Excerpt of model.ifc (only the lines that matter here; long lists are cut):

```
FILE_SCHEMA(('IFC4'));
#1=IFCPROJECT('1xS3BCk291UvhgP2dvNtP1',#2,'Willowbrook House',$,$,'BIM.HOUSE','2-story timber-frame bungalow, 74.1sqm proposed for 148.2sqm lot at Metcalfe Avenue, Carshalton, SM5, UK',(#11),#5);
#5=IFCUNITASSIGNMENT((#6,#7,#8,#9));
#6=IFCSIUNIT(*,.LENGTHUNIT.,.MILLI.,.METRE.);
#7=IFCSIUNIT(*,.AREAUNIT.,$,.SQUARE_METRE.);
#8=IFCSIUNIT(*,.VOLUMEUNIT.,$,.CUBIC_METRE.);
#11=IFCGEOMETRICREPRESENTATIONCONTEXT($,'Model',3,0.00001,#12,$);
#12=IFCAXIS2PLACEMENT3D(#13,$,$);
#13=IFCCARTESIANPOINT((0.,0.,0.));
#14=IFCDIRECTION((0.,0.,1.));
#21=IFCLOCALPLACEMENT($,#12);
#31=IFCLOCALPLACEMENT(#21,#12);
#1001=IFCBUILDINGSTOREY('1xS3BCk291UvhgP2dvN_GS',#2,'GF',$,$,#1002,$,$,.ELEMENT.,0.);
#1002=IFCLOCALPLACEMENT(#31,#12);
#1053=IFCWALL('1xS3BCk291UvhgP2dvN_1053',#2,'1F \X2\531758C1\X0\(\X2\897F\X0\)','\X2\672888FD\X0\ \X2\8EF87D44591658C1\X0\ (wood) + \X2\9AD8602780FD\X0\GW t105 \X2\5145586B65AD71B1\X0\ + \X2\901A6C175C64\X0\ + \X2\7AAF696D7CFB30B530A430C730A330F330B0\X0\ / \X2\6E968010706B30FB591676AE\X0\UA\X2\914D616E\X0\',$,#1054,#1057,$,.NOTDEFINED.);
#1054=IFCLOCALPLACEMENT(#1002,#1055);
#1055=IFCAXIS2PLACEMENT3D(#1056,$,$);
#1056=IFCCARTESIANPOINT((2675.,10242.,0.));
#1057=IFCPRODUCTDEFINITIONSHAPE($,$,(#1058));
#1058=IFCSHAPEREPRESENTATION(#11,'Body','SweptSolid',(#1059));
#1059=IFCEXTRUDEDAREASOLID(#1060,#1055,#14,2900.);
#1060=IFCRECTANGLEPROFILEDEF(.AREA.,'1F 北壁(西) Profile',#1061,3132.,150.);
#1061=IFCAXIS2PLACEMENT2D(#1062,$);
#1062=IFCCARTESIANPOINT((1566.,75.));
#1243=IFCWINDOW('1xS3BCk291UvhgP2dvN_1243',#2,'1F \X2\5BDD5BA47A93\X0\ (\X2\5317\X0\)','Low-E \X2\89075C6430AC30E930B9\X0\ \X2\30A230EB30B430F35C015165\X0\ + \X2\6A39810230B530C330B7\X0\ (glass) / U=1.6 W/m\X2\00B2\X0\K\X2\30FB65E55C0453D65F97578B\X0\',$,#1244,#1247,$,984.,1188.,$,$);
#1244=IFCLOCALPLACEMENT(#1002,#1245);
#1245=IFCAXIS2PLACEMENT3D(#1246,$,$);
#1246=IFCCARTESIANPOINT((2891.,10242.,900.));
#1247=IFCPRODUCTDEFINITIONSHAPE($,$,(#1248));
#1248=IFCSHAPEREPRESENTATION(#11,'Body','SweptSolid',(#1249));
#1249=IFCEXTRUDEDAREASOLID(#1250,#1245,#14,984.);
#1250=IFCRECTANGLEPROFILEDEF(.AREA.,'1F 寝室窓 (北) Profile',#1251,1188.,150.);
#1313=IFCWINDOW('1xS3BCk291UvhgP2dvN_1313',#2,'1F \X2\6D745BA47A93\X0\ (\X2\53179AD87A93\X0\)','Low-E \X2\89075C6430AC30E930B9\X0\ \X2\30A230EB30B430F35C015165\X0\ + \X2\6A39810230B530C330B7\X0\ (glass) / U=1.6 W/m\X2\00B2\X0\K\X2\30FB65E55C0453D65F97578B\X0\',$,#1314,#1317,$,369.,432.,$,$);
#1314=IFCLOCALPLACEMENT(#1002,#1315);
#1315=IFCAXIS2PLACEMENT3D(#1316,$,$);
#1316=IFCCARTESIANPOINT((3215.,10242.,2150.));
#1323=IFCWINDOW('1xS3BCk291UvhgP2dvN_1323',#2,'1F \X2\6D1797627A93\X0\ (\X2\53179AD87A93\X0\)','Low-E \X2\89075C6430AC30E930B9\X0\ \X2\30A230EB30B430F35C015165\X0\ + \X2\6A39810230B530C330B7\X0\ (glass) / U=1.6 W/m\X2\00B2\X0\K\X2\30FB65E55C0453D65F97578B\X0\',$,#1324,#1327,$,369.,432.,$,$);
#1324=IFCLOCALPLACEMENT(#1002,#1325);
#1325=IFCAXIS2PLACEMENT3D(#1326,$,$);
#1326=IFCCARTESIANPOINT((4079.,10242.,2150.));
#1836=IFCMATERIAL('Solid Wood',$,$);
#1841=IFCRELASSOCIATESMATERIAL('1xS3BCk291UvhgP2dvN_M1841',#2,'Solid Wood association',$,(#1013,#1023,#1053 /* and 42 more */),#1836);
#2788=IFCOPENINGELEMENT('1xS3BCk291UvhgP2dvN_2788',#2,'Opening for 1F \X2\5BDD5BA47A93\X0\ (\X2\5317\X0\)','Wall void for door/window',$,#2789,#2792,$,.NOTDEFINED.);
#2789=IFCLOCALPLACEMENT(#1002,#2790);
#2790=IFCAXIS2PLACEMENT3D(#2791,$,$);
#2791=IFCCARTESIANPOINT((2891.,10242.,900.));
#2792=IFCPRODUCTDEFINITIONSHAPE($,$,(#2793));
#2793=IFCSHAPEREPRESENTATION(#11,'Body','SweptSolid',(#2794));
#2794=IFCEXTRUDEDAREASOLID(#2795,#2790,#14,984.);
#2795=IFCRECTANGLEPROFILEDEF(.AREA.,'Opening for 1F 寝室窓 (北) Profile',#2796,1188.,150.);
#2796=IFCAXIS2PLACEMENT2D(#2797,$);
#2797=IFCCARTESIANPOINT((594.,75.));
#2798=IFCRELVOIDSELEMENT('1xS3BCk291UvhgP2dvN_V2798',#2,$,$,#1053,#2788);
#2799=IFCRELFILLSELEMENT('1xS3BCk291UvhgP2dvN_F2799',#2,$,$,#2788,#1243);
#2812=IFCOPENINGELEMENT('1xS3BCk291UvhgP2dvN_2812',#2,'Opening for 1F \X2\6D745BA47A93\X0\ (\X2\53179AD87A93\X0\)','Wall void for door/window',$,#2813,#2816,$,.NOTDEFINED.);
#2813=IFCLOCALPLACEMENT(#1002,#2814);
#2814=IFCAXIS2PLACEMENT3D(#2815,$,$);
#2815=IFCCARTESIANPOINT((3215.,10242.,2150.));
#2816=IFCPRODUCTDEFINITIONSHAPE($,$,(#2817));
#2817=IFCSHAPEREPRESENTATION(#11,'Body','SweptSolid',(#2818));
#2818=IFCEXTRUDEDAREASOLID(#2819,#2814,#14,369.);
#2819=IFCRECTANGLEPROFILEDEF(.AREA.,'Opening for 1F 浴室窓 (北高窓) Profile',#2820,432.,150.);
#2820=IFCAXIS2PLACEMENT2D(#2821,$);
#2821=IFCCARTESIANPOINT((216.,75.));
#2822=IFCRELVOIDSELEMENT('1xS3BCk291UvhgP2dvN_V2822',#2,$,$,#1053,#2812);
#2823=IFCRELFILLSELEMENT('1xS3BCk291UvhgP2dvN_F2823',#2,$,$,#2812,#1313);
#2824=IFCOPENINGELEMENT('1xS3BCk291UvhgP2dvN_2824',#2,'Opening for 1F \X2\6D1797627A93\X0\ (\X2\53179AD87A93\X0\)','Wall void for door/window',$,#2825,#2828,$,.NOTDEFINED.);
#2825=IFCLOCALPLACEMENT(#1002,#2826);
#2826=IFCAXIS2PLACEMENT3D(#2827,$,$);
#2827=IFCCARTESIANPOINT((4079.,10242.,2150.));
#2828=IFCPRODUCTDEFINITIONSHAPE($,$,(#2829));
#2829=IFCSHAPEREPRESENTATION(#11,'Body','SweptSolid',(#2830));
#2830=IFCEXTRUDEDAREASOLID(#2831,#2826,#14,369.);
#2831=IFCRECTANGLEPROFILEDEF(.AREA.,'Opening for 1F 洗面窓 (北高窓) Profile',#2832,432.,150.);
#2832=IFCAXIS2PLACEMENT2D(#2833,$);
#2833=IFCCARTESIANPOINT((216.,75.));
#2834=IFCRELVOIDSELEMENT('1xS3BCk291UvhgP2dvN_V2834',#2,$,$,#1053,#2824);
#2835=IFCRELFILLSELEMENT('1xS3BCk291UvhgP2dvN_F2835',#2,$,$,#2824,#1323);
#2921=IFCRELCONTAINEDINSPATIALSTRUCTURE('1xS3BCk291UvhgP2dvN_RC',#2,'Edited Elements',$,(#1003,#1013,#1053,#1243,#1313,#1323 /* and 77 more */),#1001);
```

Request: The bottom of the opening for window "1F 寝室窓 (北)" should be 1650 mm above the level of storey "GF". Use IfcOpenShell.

```python
import numpy as np
import ifcopenshell
import ifcopenshell.api.geometry
import ifcopenshell.geom
import ifcopenshell.util.element
import ifcopenshell.util.placement
import ifcopenshell.util.shape
import ifcopenshell.util.unit

model = ifcopenshell.open("model.ifc")
unit_scale = ifcopenshell.util.unit.calculate_unit_scale(model)

window = model.by_id(1243)
opening = window.FillsVoids[0].RelatingOpeningElement
storey = ifcopenshell.util.element.get_container(window, ifc_class="IfcBuildingStorey")
level = ifcopenshell.util.placement.get_local_placement(storey.ObjectPlacement)[2, 3]

# The opening's origin need not be at the sill, so measure its lowest point.
shape = ifcopenshell.geom.create_shape(ifcopenshell.geom.settings(), opening)
bottom = ifcopenshell.util.shape.get_shape_bottom_elevation(shape, shape.geometry) / unit_scale
dz = level + 1.65 / unit_scale - bottom

shift = np.array([0.0, 0.0, dz])
# The window is not placed relative to its opening, so move both.
for product in (opening, window):
    matrix = ifcopenshell.util.placement.get_local_placement(product.ObjectPlacement)
    matrix[:3, 3] += shift
    ifcopenshell.api.geometry.edit_object_placement(model, product=product, matrix=matrix, is_si=False)

print(f"moved by {dz * unit_scale:+.3f} m")

model.write("model_edited.ifc")
```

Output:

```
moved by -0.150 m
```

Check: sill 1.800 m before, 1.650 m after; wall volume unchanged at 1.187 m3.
